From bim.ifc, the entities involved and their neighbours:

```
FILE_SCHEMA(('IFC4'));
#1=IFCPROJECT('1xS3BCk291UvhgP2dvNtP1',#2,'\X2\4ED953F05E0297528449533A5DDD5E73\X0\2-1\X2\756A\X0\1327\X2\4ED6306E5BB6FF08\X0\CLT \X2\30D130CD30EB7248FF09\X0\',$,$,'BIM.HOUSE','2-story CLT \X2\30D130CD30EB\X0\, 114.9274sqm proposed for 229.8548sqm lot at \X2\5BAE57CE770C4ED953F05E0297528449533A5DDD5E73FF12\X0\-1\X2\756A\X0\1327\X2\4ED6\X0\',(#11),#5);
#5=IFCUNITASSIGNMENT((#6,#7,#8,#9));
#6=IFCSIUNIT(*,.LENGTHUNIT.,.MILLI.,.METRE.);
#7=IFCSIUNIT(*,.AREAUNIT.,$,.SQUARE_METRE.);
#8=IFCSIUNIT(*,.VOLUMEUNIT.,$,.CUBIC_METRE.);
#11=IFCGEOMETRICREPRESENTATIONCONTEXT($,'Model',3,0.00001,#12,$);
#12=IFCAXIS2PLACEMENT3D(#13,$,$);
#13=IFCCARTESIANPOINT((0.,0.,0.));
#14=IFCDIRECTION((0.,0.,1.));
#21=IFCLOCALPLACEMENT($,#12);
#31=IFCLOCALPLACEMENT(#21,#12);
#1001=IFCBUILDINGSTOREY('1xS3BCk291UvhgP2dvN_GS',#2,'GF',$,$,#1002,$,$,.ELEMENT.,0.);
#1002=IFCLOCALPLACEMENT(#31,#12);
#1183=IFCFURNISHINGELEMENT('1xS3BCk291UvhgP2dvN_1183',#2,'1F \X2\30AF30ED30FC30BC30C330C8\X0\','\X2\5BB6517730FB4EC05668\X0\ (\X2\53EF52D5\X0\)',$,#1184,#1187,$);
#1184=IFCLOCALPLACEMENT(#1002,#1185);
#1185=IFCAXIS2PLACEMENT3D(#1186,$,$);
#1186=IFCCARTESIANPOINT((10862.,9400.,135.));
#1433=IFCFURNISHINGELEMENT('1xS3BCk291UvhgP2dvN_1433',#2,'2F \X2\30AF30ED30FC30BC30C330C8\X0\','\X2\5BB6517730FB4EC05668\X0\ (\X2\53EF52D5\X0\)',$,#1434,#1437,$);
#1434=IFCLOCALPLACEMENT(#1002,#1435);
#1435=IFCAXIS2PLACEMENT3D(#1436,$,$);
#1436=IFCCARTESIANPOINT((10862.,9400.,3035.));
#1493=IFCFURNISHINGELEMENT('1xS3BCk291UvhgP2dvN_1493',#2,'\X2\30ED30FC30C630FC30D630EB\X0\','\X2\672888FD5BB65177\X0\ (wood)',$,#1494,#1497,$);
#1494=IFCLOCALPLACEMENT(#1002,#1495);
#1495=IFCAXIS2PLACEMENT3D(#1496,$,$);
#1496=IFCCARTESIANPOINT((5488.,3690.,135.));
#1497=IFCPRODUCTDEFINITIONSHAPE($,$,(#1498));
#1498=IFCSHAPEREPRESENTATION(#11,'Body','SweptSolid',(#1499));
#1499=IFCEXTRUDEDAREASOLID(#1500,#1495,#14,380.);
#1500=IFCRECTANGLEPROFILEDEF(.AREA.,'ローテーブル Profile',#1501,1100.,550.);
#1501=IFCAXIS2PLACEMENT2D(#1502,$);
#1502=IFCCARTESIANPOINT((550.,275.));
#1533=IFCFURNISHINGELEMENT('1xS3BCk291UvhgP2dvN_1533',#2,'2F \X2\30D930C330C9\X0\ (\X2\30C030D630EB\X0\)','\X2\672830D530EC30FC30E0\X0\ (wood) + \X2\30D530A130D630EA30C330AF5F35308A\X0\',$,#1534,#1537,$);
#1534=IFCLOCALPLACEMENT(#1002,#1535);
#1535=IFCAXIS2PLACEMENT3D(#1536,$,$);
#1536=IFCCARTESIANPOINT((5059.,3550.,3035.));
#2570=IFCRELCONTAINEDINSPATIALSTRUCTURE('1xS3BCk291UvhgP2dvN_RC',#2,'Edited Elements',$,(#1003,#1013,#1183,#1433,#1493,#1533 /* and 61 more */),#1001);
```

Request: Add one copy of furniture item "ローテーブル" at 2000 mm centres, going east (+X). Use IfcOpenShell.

```python
import numpy as np
import ifcopenshell
import ifcopenshell.api.geometry
import ifcopenshell.api.root
import ifcopenshell.util.element
import ifcopenshell.util.placement

model = ifcopenshell.open("bim.ifc")


def reuse_history(source, copy):
    """copy_class also copies each property set's owner history, people and application; keep the originals."""
    for rel in copy.IsDefinedBy:
        if rel.is_a("IfcRelDefinesByProperties") and (history := rel.RelatingPropertyDefinition.OwnerHistory):
            rel.RelatingPropertyDefinition.OwnerHistory = source.OwnerHistory
            ifcopenshell.util.element.remove_deep2(model, history)


source = model.by_guid("1xS3BCk291UvhgP2dvN_1493")
base = ifcopenshell.util.placement.get_local_placement(source.ObjectPlacement)
step = np.array([1.0, 0.0, 0.0]) * 2000.0

for i in range(1, 2):
    copy = ifcopenshell.api.root.copy_class(model, product=source)
    copy.Representation = ifcopenshell.util.element.copy_deep(
        model, source.Representation, exclude=["IfcGeometricRepresentationContext", "IfcRepresentationMap"]
    )
    reuse_history(source, copy)
    matrix = base.copy()
    matrix[:3, 3] += i * step
    print("added at", matrix[:3, 3].round(3) + 0.0)
    ifcopenshell.api.geometry.edit_object_placement(model, product=copy, matrix=matrix, is_si=False)

model.write("bim-out.ifc")
```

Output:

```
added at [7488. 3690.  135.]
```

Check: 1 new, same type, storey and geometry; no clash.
